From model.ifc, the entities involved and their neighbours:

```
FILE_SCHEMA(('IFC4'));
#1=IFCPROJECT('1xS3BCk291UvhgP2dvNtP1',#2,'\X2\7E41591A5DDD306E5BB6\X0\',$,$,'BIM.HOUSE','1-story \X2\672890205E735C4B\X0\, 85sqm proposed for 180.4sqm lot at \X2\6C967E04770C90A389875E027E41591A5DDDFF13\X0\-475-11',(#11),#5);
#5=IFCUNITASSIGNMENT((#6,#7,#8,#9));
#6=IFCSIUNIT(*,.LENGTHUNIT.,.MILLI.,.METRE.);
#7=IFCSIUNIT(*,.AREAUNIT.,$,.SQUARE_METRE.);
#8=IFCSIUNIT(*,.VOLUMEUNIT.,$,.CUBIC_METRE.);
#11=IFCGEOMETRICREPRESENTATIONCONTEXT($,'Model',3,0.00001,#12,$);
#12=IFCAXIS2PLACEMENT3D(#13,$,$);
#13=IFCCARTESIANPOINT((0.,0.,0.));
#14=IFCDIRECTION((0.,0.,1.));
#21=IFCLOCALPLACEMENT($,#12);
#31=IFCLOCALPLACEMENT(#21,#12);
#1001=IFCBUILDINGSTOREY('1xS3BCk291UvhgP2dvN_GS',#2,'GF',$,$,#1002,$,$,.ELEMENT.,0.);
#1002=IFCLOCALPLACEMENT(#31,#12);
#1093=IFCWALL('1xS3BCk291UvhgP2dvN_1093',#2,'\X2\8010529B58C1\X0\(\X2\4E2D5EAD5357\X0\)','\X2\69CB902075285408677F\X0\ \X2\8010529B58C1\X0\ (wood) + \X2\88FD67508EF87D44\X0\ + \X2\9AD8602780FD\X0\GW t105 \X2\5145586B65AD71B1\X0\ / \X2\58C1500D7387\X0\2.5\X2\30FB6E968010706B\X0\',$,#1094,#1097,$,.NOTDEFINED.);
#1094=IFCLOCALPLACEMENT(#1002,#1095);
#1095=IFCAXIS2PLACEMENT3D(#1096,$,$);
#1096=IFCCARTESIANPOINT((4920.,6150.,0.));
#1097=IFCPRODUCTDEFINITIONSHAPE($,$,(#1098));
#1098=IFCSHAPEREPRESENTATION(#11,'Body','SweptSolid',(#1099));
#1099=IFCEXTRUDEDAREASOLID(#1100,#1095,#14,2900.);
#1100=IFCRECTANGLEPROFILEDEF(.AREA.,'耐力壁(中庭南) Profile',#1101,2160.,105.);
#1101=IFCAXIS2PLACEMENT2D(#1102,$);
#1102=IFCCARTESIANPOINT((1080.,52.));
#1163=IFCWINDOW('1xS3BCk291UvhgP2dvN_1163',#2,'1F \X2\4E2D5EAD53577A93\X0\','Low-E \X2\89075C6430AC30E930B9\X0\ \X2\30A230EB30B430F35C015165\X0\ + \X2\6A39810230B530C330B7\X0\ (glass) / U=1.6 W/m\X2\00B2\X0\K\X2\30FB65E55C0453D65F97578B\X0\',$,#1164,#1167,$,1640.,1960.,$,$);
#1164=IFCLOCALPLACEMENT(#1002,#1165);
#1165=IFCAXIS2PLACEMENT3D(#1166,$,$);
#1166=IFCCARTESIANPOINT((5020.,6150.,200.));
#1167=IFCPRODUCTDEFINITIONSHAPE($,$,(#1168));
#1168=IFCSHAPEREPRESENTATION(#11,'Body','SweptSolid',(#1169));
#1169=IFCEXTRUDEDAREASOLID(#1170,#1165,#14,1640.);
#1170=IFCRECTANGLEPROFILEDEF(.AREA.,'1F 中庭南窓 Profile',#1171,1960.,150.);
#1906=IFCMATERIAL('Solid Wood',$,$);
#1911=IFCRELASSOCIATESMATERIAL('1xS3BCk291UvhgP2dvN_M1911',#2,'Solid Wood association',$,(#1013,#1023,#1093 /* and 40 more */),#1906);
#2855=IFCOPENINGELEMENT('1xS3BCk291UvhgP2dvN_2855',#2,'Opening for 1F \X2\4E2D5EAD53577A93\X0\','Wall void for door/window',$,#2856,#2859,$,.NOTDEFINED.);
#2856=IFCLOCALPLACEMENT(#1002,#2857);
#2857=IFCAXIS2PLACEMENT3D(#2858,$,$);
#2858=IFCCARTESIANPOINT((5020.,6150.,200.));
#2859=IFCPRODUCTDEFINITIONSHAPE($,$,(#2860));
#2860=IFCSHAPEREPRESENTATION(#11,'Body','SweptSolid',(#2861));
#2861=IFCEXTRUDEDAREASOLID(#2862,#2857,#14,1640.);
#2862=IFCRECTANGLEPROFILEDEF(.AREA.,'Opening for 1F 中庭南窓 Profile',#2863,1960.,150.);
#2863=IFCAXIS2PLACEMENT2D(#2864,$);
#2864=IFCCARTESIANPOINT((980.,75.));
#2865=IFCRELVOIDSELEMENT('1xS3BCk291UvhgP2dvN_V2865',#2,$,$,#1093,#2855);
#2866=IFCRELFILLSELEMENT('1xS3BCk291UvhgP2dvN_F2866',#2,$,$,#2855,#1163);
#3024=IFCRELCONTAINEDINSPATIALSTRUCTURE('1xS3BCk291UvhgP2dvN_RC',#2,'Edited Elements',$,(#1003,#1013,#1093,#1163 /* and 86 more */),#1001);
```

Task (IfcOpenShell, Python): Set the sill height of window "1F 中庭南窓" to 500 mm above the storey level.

```python
import numpy as np
import ifcopenshell
import ifcopenshell.api.geometry
import ifcopenshell.geom
import ifcopenshell.util.element
import ifcopenshell.util.placement
import ifcopenshell.util.shape
import ifcopenshell.util.unit

model = ifcopenshell.open("model.ifc")
unit_scale = ifcopenshell.util.unit.calculate_unit_scale(model)

window = model.by_id(1163)
opening = window.FillsVoids[0].RelatingOpeningElement
storey = ifcopenshell.util.element.get_container(window, ifc_class="IfcBuildingStorey")
level = ifcopenshell.util.placement.get_local_placement(storey.ObjectPlacement)[2, 3]

# The opening's origin need not be at the sill, so measure its lowest point.
shape = ifcopenshell.geom.create_shape(ifcopenshell.geom.settings(), opening)
bottom = ifcopenshell.util.shape.get_shape_bottom_elevation(shape, shape.geometry) / unit_scale
dz = level + 0.5 / unit_scale - bottom

shift = np.array([0.0, 0.0, dz])
# The window is not placed relative to its opening, so move both.
for product in (opening, window):
    matrix = ifcopenshell.util.placement.get_local_placement(product.ObjectPlacement)
    matrix[:3, 3] += shift
    ifcopenshell.api.geometry.edit_object_placement(model, product=product, matrix=matrix, is_si=False)

print(f"moved by {dz * unit_scale:+.3f} m")

model.write("model-out.ifc")
```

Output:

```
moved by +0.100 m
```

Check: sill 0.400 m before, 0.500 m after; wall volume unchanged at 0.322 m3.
